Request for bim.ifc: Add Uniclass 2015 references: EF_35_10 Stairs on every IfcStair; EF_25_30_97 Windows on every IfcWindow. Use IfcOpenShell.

First a look at what the model holds.

```python
import ifcopenshell

model = ifcopenshell.open("bim.ifc")
print(model.schema)
print("classifications:", [c.Name for c in model.by_type("IfcClassification")])
for ifc_class in ("IfcDoor", "IfcRoof", "IfcStair", "IfcWall", "IfcWindow"):
    print(ifc_class, len(model.by_type(ifc_class)))
```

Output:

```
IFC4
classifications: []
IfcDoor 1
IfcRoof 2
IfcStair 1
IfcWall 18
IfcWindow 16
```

```python
import ifcopenshell
import ifcopenshell.api.classification

model = ifcopenshell.open("bim.ifc")

system = ifcopenshell.api.classification.add_classification(model, classification="Uniclass 2015")

codes = {
    "IfcStair": ("EF_35_10", "Stairs"),
    "IfcWindow": ("EF_25_30_97", "Windows"),
}
for ifc_class, (code, name) in codes.items():
    products = model.by_type(ifc_class)
    ifcopenshell.api.classification.add_reference(
        model, products=products, classification=system, identification=code, name=name
    )
    print(code, len(products))

model.write("bim_rev.ifc")
```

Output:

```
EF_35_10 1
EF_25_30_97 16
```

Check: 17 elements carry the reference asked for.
